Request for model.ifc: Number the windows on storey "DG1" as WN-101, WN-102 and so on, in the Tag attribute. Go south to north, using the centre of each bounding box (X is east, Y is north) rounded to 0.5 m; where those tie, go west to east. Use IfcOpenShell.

First a look at what the model holds.

```python
import ifcopenshell
import ifcopenshell.util.element
import ifcopenshell.util.placement

model = ifcopenshell.open("model.ifc")
print(model.schema)
storey = next(s for s in model.by_type("IfcBuildingStorey") if s.Name == "DG1")
windows = [e for e in ifcopenshell.util.element.get_decomposition(storey) if e.is_a("IfcWindow")]
for e in sorted(windows, key=lambda e: e.id()):
    origin = ifcopenshell.util.placement.get_local_placement(e.ObjectPlacement)[:3, 3]
    print(e.id(), e.Tag, e.Name, origin.round(2) + 0.0, sep=" | ")
```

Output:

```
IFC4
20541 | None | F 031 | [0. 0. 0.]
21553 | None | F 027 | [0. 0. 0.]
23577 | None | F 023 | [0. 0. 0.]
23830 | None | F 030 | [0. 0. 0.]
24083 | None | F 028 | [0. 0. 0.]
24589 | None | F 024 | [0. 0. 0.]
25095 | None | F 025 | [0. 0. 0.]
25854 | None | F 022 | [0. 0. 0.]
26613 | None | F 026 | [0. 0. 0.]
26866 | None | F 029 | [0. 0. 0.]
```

```python
import ifcopenshell
import ifcopenshell.geom
import ifcopenshell.util.element
import ifcopenshell.util.shape

model = ifcopenshell.open("model.ifc")
settings = ifcopenshell.geom.settings()
settings.set("use-world-coords", True)


def centre(element):
    shape = ifcopenshell.geom.create_shape(settings, element)
    return ifcopenshell.util.shape.get_bbox_centroid(shape.geometry)


storey = next(s for s in model.by_type("IfcBuildingStorey") if s.Name == "DG1")
windows = [e for e in ifcopenshell.util.element.get_decomposition(storey) if e.is_a("IfcWindow")]

# Insertion points can sit at a corner or the storey origin, so sort by the geometry (in metres).
centres = {e: centre(e) for e in windows}
windows.sort(key=lambda e: (round(centres[e][1] / 0.5), centres[e][0]))

for i, e in enumerate(windows, start=1):
    number = f"WN-1{i:02d}"
    e.Tag = number
    print(e.id(), number)

model.write("model-out.ifc")
```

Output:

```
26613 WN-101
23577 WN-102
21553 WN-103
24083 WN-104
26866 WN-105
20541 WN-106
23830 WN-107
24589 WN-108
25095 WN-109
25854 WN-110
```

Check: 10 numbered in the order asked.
